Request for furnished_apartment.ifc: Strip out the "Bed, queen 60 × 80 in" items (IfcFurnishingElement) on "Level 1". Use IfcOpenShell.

First a look at what the model holds.

```python
import ifcopenshell
import ifcopenshell.util.element

model = ifcopenshell.open("furnished_apartment.ifc")
print(model.schema)
storey = next(s for s in model.by_type("IfcBuildingStorey") if s.Name == "Level 1")
furniture = [e for e in ifcopenshell.util.element.get_decomposition(storey) if e.is_a("IfcFurnishingElement")]
seen = {}
for e in furniture:
    element_type = ifcopenshell.util.element.get_type(e)
    name = element_type.Name if element_type not in (None, e) else None
    seen[name] = seen.get(name, 0) + 1
for name, count in sorted(seen.items(), key=str):
    print(count, "x", name)
```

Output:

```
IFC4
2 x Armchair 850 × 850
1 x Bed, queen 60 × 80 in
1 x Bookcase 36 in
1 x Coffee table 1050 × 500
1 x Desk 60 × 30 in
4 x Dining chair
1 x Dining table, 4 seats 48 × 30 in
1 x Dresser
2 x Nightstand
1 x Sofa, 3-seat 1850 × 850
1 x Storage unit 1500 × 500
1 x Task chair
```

```python
import ifcopenshell
import ifcopenshell.api.root
import ifcopenshell.util.element

model = ifcopenshell.open("furnished_apartment.ifc")

storey = next(s for s in model.by_type("IfcBuildingStorey") if s.Name == "Level 1")
furniture = [e for e in ifcopenshell.util.element.get_decomposition(storey) if e.is_a("IfcFurnishingElement")]
targets = [e for e in furniture if (t := ifcopenshell.util.element.get_type(e)) not in (None, e) and t.Name == "Bed, queen 60 × 80 in"]

for e in targets:
    ifcopenshell.api.root.remove_product(model, product=e)
print(len(targets), "removed")

model.write("furnished_apartment_rev.ifc")
```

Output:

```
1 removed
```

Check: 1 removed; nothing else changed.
